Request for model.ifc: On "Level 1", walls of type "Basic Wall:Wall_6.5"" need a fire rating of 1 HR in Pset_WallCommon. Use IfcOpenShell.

First a look at what the model holds.

```python
import ifcopenshell
import ifcopenshell.util.element

model = ifcopenshell.open("model.ifc")
print(model.schema)
storey = next(s for s in model.by_type("IfcBuildingStorey") if s.Name == "Level 1")
walls = [e for e in ifcopenshell.util.element.get_decomposition(storey) if e.is_a("IfcWall")]
seen = {}
for e in walls:
    element_type = ifcopenshell.util.element.get_type(e)
    key = (element_type.Name if element_type != e and element_type else None, ifcopenshell.util.element.get_pset(e, "Pset_WallCommon", "FireRating"))
    seen[key] = seen.get(key, 0) + 1
for (name, value), count in sorted(seen.items(), key=str):
    print(count, "x", name, "|", value)
```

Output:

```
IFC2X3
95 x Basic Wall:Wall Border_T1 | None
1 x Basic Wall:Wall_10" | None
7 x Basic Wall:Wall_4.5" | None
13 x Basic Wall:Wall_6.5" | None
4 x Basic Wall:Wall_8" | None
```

```python
import ifcopenshell
import ifcopenshell.api.pset
import ifcopenshell.util.element

model = ifcopenshell.open("model.ifc")

storey = next(s for s in model.by_type("IfcBuildingStorey") if s.Name == "Level 1")
walls = [e for e in ifcopenshell.util.element.get_decomposition(storey) if e.is_a("IfcWall")]

count = 0
for e in walls:
    element_type = ifcopenshell.util.element.get_type(e)
    if element_type in (None, e) or element_type.Name != 'Basic Wall:Wall_6.5"':
        continue
    # add_pset returns the element's existing set when there is one.
    pset = ifcopenshell.api.pset.add_pset(model, product=e, name="Pset_WallCommon")
    ifcopenshell.api.pset.edit_pset(model, pset=pset, properties={"FireRating": "1 HR"})
    count += 1

print(count, "walls updated")

model.write("model_edited.ifc")
```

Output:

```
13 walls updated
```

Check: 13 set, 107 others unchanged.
